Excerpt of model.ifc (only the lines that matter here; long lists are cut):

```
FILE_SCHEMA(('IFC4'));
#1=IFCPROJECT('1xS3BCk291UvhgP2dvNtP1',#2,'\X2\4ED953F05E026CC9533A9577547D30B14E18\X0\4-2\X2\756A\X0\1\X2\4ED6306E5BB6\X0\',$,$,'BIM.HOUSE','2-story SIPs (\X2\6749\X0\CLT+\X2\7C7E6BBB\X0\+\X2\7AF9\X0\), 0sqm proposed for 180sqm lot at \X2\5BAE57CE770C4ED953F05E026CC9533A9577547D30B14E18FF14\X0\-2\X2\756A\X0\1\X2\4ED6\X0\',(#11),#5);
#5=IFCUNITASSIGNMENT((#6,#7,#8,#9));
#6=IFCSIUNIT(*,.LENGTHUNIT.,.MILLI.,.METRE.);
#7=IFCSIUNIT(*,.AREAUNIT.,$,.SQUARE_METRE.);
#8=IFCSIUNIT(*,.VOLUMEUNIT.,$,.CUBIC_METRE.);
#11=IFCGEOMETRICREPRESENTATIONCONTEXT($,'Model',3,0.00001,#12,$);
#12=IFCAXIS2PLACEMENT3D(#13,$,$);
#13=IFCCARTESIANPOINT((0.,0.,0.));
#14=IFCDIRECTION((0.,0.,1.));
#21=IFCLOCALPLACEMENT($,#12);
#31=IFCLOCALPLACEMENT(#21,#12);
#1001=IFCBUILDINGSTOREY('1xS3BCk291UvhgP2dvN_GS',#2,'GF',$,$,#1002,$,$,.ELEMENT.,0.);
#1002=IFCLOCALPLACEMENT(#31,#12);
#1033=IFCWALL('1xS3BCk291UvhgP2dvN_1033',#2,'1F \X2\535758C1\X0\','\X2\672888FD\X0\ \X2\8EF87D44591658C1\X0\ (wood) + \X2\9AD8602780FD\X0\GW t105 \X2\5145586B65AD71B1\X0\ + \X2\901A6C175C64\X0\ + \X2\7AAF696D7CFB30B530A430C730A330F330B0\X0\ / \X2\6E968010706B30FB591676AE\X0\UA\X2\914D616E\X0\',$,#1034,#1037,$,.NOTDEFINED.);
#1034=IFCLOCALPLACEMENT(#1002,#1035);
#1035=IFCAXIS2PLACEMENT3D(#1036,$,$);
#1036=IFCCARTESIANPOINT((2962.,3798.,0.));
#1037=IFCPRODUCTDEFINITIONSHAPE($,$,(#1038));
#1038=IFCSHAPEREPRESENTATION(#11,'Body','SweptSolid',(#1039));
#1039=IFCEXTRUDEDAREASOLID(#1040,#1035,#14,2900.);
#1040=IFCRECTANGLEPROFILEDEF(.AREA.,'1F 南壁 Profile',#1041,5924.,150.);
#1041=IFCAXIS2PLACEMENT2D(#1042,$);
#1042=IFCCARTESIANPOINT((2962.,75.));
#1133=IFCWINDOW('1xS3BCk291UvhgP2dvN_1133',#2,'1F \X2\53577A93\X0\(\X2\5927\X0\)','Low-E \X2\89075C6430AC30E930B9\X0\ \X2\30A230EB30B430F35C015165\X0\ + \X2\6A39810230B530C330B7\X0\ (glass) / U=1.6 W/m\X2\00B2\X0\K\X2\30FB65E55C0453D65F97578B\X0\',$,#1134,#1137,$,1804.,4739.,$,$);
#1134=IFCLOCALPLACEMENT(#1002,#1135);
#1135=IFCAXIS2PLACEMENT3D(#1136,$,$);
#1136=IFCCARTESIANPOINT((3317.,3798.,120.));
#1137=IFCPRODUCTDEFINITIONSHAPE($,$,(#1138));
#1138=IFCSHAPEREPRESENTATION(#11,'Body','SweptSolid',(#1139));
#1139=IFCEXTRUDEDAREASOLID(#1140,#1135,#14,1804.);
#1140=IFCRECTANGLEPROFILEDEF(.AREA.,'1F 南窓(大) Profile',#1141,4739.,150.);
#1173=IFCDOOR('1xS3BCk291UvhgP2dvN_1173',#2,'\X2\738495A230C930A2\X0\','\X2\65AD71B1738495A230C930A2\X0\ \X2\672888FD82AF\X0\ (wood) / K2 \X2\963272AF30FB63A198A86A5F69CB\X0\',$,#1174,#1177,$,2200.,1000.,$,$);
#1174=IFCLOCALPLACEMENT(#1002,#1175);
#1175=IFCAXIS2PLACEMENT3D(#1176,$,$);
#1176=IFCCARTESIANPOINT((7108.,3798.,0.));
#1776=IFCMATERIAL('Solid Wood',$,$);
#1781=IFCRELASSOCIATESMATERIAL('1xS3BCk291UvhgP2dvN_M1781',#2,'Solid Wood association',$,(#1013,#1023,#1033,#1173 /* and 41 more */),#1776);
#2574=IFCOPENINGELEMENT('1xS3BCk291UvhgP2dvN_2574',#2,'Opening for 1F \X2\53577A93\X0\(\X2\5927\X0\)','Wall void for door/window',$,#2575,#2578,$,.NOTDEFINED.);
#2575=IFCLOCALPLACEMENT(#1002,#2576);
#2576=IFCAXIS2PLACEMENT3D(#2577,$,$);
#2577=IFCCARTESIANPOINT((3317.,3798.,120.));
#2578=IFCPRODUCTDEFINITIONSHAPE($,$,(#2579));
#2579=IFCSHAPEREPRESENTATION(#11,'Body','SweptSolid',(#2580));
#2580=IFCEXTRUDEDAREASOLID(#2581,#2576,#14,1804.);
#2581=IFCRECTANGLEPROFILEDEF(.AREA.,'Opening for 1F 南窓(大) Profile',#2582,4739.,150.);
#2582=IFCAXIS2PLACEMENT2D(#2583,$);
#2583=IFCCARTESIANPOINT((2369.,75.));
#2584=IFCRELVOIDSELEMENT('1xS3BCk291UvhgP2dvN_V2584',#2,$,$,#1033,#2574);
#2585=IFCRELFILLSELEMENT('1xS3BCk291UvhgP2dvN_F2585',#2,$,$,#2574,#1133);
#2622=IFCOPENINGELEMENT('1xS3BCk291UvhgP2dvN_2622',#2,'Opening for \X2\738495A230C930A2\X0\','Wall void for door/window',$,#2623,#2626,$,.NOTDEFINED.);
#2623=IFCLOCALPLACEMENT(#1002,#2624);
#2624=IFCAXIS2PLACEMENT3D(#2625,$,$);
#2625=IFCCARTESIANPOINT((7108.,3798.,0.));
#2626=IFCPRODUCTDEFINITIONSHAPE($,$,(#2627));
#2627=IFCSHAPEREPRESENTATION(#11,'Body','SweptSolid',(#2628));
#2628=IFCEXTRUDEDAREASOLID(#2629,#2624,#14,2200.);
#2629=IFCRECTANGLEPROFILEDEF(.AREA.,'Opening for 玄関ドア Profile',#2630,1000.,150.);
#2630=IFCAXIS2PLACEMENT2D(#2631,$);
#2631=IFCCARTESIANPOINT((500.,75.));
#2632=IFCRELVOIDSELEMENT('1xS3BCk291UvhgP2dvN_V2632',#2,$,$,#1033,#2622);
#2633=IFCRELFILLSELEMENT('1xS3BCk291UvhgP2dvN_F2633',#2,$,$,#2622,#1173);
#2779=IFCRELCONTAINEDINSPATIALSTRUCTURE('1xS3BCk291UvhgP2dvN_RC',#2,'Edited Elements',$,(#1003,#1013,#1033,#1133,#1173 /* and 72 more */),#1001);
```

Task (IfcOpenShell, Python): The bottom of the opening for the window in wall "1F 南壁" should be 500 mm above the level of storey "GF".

```python
import numpy as np
import ifcopenshell
import ifcopenshell.api.geometry
import ifcopenshell.geom
import ifcopenshell.util.element
import ifcopenshell.util.placement
import ifcopenshell.util.shape
import ifcopenshell.util.unit

model = ifcopenshell.open("model.ifc")
unit_scale = ifcopenshell.util.unit.calculate_unit_scale(model)

window = model.by_id(1133)
opening = window.FillsVoids[0].RelatingOpeningElement
storey = ifcopenshell.util.element.get_container(window, ifc_class="IfcBuildingStorey")
level = ifcopenshell.util.placement.get_local_placement(storey.ObjectPlacement)[2, 3]

# The opening's origin need not be at the sill, so measure its lowest point.
shape = ifcopenshell.geom.create_shape(ifcopenshell.geom.settings(), opening)
bottom = ifcopenshell.util.shape.get_shape_bottom_elevation(shape, shape.geometry) / unit_scale
dz = level + 0.5 / unit_scale - bottom

shift = np.array([0.0, 0.0, dz])
# The window is not placed relative to its opening, so move both.
for product in (opening, window):
    matrix = ifcopenshell.util.placement.get_local_placement(product.ObjectPlacement)
    matrix[:3, 3] += shift
    ifcopenshell.api.geometry.edit_object_placement(model, product=product, matrix=matrix, is_si=False)

print(f"moved by {dz * unit_scale:+.3f} m")

model.write("model_edited.ifc")
```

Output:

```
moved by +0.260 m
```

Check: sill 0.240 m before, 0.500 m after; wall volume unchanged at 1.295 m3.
